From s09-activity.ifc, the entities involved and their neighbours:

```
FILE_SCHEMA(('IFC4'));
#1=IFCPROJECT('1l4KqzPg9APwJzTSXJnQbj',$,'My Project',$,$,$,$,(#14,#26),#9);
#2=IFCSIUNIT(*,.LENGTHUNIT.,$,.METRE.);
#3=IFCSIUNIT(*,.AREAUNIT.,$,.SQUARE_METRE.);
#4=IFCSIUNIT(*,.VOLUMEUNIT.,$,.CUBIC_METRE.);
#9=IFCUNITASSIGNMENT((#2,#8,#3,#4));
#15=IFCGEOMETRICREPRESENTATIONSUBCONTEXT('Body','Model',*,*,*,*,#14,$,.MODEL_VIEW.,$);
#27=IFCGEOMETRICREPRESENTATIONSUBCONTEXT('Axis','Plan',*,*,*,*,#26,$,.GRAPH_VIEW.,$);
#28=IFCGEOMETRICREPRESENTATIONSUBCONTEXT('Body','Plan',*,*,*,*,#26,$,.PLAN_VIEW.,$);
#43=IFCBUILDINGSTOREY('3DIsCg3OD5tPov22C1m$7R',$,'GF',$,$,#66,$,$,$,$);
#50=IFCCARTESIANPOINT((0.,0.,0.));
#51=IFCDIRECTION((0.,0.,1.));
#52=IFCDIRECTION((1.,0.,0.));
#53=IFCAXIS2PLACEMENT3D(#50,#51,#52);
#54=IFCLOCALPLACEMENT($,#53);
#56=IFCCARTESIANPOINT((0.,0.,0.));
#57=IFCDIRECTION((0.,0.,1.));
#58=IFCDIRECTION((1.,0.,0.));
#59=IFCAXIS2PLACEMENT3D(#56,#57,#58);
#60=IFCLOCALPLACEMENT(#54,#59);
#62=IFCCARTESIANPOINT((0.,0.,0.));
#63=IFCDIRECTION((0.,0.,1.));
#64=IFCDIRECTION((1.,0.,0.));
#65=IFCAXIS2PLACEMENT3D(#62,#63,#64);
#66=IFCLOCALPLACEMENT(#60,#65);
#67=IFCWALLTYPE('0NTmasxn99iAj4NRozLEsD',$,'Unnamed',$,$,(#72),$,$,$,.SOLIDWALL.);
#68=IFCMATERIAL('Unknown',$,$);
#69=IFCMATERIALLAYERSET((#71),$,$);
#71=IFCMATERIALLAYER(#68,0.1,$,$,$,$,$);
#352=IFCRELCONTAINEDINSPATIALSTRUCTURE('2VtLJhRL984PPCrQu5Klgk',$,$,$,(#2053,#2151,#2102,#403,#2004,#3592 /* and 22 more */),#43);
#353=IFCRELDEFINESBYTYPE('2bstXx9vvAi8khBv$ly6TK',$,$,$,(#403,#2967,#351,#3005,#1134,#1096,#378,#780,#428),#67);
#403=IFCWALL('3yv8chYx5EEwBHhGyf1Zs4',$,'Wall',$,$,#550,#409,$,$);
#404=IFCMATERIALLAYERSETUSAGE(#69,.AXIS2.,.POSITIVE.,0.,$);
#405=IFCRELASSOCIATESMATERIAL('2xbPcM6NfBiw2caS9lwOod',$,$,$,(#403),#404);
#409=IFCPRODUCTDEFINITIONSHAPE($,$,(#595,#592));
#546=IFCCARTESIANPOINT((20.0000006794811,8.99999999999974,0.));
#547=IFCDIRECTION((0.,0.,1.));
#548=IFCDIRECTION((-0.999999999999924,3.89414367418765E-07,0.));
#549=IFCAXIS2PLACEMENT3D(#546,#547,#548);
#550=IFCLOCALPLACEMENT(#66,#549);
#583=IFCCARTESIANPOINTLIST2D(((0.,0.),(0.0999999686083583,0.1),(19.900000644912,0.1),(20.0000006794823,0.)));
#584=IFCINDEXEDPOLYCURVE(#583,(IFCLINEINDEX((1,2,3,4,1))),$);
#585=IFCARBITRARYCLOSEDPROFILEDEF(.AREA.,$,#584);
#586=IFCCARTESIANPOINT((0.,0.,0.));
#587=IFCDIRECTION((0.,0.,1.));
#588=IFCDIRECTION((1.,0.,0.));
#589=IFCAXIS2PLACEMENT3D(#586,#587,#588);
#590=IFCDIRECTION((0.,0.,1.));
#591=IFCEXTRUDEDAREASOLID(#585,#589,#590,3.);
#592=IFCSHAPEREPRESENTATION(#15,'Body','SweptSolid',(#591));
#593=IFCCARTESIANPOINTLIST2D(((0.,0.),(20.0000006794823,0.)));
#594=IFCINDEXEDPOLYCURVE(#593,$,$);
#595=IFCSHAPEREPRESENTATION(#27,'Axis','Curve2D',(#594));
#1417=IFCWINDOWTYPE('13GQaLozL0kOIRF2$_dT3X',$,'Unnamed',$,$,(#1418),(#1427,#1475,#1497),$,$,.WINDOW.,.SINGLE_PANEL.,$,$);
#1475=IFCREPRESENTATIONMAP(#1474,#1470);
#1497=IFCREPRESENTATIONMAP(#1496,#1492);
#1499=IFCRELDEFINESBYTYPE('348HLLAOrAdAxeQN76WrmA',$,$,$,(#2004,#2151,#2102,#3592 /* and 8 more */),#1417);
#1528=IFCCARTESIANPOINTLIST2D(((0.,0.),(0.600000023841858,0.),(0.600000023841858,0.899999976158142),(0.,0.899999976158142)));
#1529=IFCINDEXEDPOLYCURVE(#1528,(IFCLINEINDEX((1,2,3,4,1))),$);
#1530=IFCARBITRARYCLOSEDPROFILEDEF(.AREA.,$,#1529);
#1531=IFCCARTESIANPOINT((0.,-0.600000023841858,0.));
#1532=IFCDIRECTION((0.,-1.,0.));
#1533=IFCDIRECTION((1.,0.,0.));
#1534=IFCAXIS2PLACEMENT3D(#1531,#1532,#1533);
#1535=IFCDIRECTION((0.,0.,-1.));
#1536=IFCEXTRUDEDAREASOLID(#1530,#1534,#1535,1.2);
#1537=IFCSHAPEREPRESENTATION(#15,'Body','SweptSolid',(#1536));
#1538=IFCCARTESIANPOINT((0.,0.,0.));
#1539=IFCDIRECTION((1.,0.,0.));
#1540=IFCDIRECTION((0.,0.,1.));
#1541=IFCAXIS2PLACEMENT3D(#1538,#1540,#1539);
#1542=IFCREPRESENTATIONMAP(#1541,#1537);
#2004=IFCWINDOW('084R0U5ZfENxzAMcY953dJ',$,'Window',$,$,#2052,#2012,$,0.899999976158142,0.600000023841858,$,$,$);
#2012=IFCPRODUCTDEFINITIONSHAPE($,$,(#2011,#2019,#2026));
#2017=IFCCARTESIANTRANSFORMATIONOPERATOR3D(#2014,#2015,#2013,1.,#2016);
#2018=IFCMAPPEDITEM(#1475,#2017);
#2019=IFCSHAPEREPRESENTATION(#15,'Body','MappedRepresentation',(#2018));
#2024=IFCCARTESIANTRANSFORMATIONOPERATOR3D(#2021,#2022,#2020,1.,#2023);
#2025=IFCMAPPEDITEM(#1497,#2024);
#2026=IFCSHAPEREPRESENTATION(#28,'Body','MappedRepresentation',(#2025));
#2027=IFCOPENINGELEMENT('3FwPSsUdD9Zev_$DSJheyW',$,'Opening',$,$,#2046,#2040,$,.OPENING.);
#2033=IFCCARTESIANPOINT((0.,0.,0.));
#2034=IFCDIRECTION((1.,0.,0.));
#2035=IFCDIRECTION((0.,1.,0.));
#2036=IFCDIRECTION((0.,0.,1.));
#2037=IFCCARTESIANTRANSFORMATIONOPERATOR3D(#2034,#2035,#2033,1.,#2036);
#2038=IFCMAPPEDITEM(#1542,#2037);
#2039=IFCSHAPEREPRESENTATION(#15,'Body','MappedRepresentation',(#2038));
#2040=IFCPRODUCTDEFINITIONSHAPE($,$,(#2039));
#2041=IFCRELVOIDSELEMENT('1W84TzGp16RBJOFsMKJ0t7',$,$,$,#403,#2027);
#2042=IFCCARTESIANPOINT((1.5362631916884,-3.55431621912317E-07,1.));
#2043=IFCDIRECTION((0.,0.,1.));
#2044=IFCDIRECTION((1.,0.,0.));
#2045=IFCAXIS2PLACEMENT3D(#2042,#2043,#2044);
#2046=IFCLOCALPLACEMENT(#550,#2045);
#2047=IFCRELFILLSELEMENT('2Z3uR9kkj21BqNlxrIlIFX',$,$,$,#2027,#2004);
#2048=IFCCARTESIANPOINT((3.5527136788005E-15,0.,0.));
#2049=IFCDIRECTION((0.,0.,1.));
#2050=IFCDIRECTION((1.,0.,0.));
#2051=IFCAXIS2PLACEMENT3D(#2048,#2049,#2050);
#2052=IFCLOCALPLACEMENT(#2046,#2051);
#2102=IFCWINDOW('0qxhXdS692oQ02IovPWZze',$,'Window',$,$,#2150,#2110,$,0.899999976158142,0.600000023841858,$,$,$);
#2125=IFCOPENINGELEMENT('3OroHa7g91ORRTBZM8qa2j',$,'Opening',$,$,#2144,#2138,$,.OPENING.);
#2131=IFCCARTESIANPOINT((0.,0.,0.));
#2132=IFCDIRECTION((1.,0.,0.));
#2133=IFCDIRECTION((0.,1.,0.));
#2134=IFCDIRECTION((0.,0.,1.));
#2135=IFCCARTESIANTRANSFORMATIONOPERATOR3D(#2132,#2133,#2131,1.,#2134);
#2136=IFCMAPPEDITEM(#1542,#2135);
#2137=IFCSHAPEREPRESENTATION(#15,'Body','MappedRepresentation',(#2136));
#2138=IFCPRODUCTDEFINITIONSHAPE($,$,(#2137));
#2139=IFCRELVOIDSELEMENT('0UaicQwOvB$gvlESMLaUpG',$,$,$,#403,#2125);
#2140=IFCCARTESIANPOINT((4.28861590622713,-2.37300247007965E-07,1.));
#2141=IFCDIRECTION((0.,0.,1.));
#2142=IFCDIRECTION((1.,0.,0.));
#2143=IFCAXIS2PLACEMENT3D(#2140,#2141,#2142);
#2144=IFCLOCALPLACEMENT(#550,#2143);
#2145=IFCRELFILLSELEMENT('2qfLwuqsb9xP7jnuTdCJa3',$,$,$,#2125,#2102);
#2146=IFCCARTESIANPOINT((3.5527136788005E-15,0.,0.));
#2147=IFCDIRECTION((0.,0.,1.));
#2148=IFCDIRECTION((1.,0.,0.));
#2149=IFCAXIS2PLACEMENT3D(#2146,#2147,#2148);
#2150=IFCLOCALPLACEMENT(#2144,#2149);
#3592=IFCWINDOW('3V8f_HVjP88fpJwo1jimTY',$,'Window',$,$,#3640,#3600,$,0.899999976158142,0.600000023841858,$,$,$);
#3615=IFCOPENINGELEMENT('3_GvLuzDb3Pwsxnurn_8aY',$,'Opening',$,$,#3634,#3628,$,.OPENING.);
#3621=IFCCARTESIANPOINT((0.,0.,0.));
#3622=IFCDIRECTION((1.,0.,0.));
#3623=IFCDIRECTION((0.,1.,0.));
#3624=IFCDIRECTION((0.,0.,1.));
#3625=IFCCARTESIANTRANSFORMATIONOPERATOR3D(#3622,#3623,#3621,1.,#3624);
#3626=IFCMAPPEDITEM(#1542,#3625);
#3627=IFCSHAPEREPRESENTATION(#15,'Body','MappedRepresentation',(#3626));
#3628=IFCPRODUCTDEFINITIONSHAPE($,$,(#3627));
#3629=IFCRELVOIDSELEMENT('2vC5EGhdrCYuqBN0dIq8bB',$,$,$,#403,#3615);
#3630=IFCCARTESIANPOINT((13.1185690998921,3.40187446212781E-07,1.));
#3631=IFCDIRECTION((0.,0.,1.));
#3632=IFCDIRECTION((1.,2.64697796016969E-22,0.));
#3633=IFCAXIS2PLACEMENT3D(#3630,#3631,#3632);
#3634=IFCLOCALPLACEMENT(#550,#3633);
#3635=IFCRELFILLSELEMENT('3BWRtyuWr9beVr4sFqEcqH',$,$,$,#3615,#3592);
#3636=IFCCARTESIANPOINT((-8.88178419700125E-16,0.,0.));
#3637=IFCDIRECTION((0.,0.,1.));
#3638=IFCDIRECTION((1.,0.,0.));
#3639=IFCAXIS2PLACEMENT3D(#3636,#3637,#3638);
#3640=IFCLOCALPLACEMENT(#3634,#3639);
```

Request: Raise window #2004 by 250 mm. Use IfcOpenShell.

```python
import numpy as np
import ifcopenshell
import ifcopenshell.api.geometry
import ifcopenshell.util.placement
import ifcopenshell.util.unit

model = ifcopenshell.open("s09-activity.ifc")
unit_scale = ifcopenshell.util.unit.calculate_unit_scale(model)

window = model.by_guid("084R0U5ZfENxzAMcY953dJ")
opening = window.FillsVoids[0].RelatingOpeningElement
dz = 0.25 / unit_scale

shift = np.array([0.0, 0.0, dz])
# The window is placed relative to its opening, so it follows when the opening moves.
matrix = ifcopenshell.util.placement.get_local_placement(opening.ObjectPlacement)
matrix[:3, 3] += shift
ifcopenshell.api.geometry.edit_object_placement(
    model, product=opening, matrix=matrix, is_si=False, should_transform_children=True
)

print(f"moved by {dz * unit_scale:+.3f} m")

model.write("s09-activity_edited.ifc")
```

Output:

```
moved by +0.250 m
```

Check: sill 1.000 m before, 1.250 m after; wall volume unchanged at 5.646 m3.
